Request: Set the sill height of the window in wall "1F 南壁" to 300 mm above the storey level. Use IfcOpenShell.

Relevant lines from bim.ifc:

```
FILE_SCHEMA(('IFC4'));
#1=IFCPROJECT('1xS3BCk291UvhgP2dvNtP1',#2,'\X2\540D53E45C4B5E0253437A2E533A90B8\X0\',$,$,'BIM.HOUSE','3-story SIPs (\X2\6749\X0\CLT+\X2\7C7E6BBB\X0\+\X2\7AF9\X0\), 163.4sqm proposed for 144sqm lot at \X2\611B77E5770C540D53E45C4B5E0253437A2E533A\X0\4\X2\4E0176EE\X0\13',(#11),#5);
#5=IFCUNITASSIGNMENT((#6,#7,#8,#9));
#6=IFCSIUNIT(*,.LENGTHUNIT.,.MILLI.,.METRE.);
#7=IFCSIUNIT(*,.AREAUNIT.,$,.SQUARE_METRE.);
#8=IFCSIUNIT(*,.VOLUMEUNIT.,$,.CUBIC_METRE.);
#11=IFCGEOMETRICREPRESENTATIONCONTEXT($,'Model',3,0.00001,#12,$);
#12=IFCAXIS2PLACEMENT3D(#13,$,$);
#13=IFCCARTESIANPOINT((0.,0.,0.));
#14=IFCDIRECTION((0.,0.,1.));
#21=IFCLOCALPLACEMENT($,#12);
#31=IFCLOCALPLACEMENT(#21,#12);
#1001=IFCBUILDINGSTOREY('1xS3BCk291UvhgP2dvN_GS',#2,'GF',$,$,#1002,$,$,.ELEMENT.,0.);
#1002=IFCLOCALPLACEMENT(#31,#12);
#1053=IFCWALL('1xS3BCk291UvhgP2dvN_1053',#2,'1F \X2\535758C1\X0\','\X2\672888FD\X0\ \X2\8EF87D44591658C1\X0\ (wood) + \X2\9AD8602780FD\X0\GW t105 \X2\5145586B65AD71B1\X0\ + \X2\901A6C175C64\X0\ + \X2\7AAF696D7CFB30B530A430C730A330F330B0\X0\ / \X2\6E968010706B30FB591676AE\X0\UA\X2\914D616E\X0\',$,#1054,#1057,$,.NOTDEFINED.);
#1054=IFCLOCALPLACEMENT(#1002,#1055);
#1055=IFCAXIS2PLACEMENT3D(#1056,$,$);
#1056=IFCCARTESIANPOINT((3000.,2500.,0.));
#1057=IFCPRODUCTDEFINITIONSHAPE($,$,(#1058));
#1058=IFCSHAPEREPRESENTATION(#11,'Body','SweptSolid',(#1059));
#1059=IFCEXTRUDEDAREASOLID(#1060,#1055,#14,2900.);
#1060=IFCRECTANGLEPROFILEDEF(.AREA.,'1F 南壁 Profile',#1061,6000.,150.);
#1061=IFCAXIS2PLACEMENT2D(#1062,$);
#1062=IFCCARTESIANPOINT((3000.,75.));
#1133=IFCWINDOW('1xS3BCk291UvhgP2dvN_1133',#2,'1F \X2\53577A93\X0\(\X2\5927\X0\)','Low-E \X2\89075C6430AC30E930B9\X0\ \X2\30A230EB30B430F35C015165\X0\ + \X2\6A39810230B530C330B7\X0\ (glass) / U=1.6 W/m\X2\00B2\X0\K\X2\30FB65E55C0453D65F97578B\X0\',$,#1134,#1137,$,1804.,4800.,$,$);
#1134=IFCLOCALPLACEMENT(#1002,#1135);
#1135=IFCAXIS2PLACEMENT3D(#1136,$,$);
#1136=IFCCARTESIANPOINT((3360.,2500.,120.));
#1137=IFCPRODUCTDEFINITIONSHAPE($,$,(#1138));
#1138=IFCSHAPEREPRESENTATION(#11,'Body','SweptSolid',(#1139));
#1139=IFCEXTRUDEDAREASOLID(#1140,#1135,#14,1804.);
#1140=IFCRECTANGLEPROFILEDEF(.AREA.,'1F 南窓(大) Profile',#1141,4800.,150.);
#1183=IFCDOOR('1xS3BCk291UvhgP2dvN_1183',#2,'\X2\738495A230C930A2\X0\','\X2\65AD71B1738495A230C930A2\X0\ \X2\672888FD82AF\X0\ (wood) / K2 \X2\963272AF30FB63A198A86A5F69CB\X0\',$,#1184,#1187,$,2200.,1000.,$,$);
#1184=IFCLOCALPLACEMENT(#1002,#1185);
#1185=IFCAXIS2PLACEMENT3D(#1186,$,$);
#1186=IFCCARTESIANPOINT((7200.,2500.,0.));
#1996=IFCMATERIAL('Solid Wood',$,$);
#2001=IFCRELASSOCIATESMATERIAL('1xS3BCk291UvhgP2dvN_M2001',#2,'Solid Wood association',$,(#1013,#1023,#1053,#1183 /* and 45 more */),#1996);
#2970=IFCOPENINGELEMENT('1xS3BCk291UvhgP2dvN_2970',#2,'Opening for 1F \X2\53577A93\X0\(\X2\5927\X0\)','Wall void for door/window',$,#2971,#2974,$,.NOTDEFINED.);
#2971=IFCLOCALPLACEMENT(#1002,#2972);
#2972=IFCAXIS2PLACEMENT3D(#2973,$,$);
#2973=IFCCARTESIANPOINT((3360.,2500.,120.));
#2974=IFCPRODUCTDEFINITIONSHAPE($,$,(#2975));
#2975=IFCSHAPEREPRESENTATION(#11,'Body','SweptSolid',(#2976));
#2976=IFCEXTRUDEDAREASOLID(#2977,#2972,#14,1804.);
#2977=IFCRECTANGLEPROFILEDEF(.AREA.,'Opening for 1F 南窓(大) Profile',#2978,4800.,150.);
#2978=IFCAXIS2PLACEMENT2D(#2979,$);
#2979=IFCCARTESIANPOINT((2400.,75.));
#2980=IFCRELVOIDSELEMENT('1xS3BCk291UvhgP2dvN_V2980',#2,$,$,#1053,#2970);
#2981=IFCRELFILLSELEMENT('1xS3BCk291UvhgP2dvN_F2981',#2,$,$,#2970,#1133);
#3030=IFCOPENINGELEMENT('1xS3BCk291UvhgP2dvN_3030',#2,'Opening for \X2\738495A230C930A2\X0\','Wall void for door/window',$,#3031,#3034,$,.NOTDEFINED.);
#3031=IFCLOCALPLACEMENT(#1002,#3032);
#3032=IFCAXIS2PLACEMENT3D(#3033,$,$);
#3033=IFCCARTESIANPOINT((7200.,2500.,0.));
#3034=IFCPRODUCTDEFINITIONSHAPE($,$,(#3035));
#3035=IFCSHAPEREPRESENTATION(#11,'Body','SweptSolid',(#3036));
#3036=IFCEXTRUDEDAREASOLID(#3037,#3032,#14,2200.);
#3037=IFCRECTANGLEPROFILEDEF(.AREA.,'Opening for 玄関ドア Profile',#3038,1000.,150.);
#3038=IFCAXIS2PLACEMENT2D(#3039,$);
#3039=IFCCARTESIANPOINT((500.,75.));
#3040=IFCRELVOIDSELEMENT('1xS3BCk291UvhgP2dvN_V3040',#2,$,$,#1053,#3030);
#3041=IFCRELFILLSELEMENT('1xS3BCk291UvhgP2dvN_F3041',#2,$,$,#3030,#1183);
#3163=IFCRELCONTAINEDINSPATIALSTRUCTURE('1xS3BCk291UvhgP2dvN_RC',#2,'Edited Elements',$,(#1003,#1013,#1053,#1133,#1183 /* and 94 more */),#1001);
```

```python
import numpy as np
import ifcopenshell
import ifcopenshell.api.geometry
import ifcopenshell.geom
import ifcopenshell.util.element
import ifcopenshell.util.placement
import ifcopenshell.util.shape
import ifcopenshell.util.unit

model = ifcopenshell.open("bim.ifc")
unit_scale = ifcopenshell.util.unit.calculate_unit_scale(model)

window = model.by_id(1133)
opening = window.FillsVoids[0].RelatingOpeningElement
storey = ifcopenshell.util.element.get_container(window, ifc_class="IfcBuildingStorey")
level = ifcopenshell.util.placement.get_local_placement(storey.ObjectPlacement)[2, 3]

# The opening's origin need not be at the sill, so measure its lowest point.
shape = ifcopenshell.geom.create_shape(ifcopenshell.geom.settings(), opening)
bottom = ifcopenshell.util.shape.get_shape_bottom_elevation(shape, shape.geometry) / unit_scale
dz = level + 0.3 / unit_scale - bottom

shift = np.array([0.0, 0.0, dz])
# The window is not placed relative to its opening, so move both.
for product in (opening, window):
    matrix = ifcopenshell.util.placement.get_local_placement(product.ObjectPlacement)
    matrix[:3, 3] += shift
    ifcopenshell.api.geometry.edit_object_placement(model, product=product, matrix=matrix, is_si=False)

print(f"moved by {dz * unit_scale:+.3f} m")

model.write("bim_edited.ifc")
```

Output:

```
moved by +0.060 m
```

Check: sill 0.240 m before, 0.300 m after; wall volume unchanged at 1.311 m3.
